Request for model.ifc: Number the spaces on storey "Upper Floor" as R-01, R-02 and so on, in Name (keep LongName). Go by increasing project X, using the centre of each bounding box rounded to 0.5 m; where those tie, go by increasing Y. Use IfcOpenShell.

First a look at what the model holds.

```python
import ifcopenshell
import ifcopenshell.util.element
import ifcopenshell.util.placement

model = ifcopenshell.open("model.ifc")
print(model.schema)
storey = next(s for s in model.by_type("IfcBuildingStorey") if s.Name == "Upper Floor")
spaces = [e for e in ifcopenshell.util.element.get_decomposition(storey) if e.is_a("IfcSpace")]
for e in sorted(spaces, key=lambda e: e.id()):
    origin = ifcopenshell.util.placement.get_local_placement(e.ObjectPlacement)[:3, 3]
    print(e.id(), e.Name, e.LongName, origin.round(2) + 0.0, sep=" | ")
```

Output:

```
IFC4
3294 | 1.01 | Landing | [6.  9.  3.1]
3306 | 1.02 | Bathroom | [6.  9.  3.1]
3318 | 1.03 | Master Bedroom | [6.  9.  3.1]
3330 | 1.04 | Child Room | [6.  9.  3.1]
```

```python
import ifcopenshell
import ifcopenshell.geom
import ifcopenshell.util.element
import ifcopenshell.util.shape

model = ifcopenshell.open("model.ifc")
settings = ifcopenshell.geom.settings()
settings.set("use-world-coords", True)


def centre(element):
    shape = ifcopenshell.geom.create_shape(settings, element)
    return ifcopenshell.util.shape.get_bbox_centroid(shape.geometry)


storey = next(s for s in model.by_type("IfcBuildingStorey") if s.Name == "Upper Floor")
spaces = [e for e in ifcopenshell.util.element.get_decomposition(storey) if e.is_a("IfcSpace")]

# Insertion points can sit at a corner or the storey origin, so sort by the geometry (in metres).
centres = {e: centre(e) for e in spaces}
spaces.sort(key=lambda e: (round(centres[e][0] / 0.5), centres[e][1]))

for i, e in enumerate(spaces, start=1):
    number = f"R-{i:02d}"
    e.Name = number
    print(e.id(), number)

model.write("model_rev.ifc")
```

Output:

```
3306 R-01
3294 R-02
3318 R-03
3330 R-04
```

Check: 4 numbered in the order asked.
